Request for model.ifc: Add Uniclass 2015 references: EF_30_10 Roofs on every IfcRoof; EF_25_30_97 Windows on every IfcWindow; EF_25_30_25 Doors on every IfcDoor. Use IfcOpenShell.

First a look at what the model holds.

```python
import ifcopenshell

model = ifcopenshell.open("model.ifc")
print(model.schema)
print("classifications:", [c.Name for c in model.by_type("IfcClassification")])
for ifc_class in ("IfcDoor", "IfcRoof", "IfcStair", "IfcWall", "IfcWindow"):
    print(ifc_class, len(model.by_type(ifc_class)))
```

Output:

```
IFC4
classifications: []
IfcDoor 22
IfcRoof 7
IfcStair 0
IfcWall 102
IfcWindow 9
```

```python
import ifcopenshell
import ifcopenshell.api.classification

model = ifcopenshell.open("model.ifc")

system = ifcopenshell.api.classification.add_classification(model, classification="Uniclass 2015")

codes = {
    "IfcRoof": ("EF_30_10", "Roofs"),
    "IfcWindow": ("EF_25_30_97", "Windows"),
    "IfcDoor": ("EF_25_30_25", "Doors"),
}
for ifc_class, (code, name) in codes.items():
    products = model.by_type(ifc_class)
    ifcopenshell.api.classification.add_reference(
        model, products=products, classification=system, identification=code, name=name
    )
    print(code, len(products))

model.write("model_edited.ifc")
```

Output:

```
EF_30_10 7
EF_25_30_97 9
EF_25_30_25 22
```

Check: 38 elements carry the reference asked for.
